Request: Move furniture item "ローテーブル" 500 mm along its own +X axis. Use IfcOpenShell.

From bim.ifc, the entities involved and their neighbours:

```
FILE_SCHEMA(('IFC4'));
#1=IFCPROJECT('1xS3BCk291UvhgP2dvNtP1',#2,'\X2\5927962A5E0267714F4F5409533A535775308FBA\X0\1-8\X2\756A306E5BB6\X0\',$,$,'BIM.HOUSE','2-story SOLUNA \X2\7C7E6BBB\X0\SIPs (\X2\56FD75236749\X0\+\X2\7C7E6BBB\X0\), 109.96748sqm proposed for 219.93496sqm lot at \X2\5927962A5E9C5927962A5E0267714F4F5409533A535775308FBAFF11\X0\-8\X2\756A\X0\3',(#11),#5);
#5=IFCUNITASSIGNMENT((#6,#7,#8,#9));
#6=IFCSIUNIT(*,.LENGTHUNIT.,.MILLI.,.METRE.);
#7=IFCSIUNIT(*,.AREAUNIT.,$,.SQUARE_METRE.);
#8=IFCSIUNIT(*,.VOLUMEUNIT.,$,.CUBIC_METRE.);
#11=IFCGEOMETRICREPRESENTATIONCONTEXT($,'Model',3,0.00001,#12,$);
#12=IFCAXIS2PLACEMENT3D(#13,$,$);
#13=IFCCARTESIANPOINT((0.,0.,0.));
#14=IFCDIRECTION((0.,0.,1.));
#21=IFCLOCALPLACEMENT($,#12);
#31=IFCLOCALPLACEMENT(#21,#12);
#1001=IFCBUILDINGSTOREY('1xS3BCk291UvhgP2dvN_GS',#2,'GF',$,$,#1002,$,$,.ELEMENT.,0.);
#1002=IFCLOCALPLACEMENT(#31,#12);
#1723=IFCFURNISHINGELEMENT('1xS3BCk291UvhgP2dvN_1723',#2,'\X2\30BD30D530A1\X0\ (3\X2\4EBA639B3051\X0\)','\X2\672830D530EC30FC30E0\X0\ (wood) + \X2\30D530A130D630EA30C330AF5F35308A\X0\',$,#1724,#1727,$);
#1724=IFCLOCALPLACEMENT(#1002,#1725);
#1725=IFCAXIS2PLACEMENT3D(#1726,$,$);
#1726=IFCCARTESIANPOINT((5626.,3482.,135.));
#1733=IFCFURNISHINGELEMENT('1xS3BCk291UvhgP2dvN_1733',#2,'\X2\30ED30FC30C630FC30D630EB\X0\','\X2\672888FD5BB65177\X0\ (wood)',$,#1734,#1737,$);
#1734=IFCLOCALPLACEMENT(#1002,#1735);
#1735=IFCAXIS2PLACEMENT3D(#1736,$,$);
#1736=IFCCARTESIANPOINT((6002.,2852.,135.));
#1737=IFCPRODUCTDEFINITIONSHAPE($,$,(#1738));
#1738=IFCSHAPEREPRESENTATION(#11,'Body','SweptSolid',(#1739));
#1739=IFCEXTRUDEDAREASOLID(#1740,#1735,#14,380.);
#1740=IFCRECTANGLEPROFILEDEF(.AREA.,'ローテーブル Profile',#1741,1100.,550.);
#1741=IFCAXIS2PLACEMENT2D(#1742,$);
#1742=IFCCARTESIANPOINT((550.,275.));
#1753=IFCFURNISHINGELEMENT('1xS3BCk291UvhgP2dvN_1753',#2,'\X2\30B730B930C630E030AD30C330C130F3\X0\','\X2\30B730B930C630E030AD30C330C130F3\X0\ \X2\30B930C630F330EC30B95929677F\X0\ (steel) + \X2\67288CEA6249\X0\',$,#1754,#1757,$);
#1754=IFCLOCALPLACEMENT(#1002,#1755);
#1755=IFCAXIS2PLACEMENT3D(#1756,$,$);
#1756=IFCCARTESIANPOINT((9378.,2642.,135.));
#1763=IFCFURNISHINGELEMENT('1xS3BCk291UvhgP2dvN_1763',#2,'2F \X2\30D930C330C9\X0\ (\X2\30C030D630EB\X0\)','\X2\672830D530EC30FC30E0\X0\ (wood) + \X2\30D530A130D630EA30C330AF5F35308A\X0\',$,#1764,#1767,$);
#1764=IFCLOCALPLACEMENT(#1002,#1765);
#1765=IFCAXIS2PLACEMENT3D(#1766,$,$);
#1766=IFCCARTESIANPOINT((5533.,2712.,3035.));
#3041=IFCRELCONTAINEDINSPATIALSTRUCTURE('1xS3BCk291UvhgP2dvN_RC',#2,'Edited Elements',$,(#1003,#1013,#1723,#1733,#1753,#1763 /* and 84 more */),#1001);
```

```python
import ifcopenshell
import ifcopenshell.api.geometry
import ifcopenshell.util.placement
import ifcopenshell.util.unit

model = ifcopenshell.open("bim.ifc")
unit_scale = ifcopenshell.util.unit.calculate_unit_scale(model)

item = model.by_guid("1xS3BCk291UvhgP2dvN_1733")
matrix = ifcopenshell.util.placement.get_local_placement(item.ObjectPlacement)
matrix[:3, 3] += matrix[:3, 0] * 0.5 / unit_scale
ifcopenshell.api.geometry.edit_object_placement(model, product=item, matrix=matrix, is_si=False)

print(ifcopenshell.util.placement.get_local_placement(item.ObjectPlacement).round(3) + 0.0)

model.write("bim_edited.ifc")
```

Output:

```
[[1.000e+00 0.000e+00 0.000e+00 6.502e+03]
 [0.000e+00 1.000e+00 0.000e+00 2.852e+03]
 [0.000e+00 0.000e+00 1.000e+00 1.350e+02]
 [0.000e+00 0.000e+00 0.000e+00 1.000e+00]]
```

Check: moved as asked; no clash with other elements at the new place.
